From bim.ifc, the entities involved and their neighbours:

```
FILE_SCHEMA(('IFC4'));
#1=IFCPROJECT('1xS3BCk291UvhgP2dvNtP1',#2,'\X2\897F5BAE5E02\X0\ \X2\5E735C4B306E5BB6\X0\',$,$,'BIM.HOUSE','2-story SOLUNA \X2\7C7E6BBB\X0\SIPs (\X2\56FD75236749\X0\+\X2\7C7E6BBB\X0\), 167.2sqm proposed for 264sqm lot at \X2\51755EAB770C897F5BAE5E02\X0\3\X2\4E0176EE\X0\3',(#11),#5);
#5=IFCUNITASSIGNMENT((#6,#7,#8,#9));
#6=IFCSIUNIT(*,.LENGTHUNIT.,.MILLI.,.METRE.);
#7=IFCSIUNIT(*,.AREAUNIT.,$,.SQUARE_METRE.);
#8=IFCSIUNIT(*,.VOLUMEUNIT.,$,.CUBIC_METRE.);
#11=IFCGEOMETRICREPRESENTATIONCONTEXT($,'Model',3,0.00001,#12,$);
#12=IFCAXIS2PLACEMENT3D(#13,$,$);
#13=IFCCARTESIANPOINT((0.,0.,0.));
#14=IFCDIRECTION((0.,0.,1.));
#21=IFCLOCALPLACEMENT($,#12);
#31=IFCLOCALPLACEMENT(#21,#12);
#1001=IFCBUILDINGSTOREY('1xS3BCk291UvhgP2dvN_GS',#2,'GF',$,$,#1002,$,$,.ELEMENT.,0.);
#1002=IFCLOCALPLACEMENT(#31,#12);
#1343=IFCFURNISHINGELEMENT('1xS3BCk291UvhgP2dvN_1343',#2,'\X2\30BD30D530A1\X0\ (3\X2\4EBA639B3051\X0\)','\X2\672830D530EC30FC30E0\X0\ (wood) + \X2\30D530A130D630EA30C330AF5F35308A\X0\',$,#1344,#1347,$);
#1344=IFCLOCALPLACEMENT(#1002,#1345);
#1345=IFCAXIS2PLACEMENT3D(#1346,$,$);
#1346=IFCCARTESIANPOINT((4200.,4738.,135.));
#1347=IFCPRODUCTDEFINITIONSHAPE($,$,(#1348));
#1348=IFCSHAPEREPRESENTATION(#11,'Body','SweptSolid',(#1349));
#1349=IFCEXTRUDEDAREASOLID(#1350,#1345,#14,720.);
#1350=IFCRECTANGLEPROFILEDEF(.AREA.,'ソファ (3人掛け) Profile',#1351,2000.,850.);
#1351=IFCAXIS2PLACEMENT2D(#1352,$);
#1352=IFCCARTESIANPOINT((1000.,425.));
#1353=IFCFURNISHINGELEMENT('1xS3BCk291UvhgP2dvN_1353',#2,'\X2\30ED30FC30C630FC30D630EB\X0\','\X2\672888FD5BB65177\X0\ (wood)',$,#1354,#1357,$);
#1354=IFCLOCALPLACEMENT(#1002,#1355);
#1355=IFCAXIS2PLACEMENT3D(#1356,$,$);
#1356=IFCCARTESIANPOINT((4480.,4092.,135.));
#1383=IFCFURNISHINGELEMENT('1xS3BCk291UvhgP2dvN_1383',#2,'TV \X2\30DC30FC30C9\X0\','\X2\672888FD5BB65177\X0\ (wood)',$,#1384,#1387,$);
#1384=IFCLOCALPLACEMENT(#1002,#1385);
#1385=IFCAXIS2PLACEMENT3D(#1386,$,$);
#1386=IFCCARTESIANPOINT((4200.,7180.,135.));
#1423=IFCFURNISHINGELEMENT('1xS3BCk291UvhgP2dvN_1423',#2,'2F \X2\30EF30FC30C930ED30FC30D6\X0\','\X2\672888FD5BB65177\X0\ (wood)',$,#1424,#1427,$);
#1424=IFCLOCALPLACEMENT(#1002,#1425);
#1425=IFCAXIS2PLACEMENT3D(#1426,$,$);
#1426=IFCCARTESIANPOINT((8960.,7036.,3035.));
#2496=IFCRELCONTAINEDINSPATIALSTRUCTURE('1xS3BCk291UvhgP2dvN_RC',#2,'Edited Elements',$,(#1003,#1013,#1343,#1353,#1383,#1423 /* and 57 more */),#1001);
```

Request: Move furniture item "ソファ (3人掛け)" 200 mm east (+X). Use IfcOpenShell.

```python
import ifcopenshell
import ifcopenshell.api.geometry
import ifcopenshell.util.placement
import ifcopenshell.util.unit

model = ifcopenshell.open("bim.ifc")
unit_scale = ifcopenshell.util.unit.calculate_unit_scale(model)

item = model.by_guid("1xS3BCk291UvhgP2dvN_1343")
matrix = ifcopenshell.util.placement.get_local_placement(item.ObjectPlacement)
matrix[0, 3] += 0.2 / unit_scale
ifcopenshell.api.geometry.edit_object_placement(model, product=item, matrix=matrix, is_si=False)

print(ifcopenshell.util.placement.get_local_placement(item.ObjectPlacement).round(3) + 0.0)

model.write("bim_edited.ifc")
```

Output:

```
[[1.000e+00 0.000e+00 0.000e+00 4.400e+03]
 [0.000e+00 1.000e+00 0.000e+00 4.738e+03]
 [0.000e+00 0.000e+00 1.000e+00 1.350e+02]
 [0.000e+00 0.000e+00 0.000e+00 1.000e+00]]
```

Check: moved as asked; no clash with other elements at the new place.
